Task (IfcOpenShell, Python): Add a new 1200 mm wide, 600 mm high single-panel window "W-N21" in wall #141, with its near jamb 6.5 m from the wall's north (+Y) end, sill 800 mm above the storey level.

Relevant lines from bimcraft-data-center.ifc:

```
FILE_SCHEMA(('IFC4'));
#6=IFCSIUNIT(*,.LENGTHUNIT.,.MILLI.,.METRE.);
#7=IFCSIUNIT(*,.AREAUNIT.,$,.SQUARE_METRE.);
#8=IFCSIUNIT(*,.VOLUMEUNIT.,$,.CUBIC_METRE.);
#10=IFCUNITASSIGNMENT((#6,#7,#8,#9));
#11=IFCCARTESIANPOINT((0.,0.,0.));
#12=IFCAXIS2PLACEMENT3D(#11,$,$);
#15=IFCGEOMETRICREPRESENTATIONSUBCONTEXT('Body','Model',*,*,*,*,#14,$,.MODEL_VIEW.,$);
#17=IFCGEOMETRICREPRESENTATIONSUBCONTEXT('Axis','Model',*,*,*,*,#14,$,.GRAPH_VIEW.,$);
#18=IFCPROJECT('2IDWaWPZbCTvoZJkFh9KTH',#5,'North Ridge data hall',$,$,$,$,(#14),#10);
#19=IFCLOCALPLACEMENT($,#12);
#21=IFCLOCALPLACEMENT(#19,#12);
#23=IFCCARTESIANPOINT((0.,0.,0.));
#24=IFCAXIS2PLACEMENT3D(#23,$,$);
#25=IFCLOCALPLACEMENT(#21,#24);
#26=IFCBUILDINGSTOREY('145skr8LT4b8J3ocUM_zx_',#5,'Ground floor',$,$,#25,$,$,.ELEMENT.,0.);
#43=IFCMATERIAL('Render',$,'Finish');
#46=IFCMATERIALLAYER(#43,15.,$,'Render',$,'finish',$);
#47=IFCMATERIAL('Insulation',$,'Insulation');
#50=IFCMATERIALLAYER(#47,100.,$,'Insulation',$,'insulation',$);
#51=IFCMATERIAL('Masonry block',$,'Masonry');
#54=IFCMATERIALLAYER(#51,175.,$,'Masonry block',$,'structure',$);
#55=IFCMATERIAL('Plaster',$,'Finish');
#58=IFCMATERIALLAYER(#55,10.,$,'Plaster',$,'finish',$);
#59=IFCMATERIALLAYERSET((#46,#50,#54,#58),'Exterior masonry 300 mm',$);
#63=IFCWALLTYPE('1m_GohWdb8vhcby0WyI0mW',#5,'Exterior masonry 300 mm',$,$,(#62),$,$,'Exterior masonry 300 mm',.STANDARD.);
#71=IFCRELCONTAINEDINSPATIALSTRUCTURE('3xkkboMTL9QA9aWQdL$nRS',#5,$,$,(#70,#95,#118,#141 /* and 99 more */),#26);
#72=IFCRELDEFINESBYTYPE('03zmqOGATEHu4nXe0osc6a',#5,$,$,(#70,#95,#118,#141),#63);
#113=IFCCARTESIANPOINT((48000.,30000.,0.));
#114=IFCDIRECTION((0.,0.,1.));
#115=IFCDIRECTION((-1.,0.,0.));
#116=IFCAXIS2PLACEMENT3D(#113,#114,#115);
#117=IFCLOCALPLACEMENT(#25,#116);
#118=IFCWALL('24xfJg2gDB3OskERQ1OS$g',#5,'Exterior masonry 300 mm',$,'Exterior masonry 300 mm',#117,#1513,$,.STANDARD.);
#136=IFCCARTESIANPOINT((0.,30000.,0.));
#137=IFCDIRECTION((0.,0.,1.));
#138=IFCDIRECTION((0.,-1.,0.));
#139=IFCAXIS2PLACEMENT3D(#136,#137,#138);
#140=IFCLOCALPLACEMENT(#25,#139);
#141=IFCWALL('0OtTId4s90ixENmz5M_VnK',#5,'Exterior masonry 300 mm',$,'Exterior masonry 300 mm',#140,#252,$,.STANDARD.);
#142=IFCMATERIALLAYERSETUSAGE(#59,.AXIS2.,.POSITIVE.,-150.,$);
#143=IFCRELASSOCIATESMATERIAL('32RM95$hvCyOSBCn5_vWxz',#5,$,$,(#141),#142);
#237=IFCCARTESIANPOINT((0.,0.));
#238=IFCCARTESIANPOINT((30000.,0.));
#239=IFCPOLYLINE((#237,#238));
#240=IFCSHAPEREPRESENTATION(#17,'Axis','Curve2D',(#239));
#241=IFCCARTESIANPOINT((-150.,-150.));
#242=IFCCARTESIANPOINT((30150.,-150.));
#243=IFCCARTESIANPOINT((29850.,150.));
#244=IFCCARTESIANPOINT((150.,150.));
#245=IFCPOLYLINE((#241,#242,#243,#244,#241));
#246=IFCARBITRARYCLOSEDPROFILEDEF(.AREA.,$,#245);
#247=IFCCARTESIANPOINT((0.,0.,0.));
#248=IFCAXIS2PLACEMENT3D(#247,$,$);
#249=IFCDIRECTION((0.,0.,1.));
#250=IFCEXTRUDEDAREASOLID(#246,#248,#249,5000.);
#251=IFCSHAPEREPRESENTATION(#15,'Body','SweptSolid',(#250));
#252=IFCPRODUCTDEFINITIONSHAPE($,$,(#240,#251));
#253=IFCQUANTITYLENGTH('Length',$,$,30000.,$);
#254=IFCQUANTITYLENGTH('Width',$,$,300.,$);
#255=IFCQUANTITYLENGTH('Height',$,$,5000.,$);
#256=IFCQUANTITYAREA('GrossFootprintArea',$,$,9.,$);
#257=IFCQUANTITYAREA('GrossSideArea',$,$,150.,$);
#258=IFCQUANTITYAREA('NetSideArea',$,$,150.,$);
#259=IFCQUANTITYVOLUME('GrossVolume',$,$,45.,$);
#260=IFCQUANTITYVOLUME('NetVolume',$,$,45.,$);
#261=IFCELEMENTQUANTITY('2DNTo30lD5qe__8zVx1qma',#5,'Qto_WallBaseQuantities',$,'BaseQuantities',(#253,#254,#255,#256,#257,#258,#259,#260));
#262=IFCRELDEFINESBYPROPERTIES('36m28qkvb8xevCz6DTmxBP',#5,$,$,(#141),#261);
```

```python
import numpy as np
import ifcopenshell
import ifcopenshell.api.feature
import ifcopenshell.api.geometry
import ifcopenshell.api.pset
import ifcopenshell.api.root
import ifcopenshell.api.spatial
import ifcopenshell.geom
import ifcopenshell.util.element
import ifcopenshell.util.placement
import ifcopenshell.util.representation
import ifcopenshell.util.shape
import ifcopenshell.util.unit

model = ifcopenshell.open("bimcraft-data-center.ifc")
unit_scale = ifcopenshell.util.unit.calculate_unit_scale(model)
area_scale = ifcopenshell.util.unit.calculate_unit_scale(model, "AREAUNIT")
volume_scale = ifcopenshell.util.unit.calculate_unit_scale(model, "VOLUMEUNIT")
settings = ifcopenshell.geom.settings()


def volume(element):
    """Net volume in cubic metres, openings subtracted."""
    shape = ifcopenshell.geom.create_shape(settings, element)
    return ifcopenshell.util.shape.get_volume(shape.geometry)


wall = model.by_id(141)
storey = ifcopenshell.util.element.get_container(wall, ifc_class="IfcBuildingStorey")
context = ifcopenshell.util.representation.get_context(model, "Model", "Body", "MODEL_VIEW")
before = volume(wall)

width, height, from_end, sill = 1.2, 0.6, 6.5, 0.8  # metres

# The wall runs along its own X axis, and the end named is its -X end.
wall_shape = ifcopenshell.geom.create_shape(settings, wall)
x, y, z = ifcopenshell.util.shape.get_vertices(wall_shape.geometry).T
start = x.min() + from_end
face, thickness = float(y.min()), float(y.max() - y.min())
wall_matrix = ifcopenshell.util.placement.get_local_placement(wall.ObjectPlacement)
level = ifcopenshell.util.placement.get_local_placement(storey.ObjectPlacement)[2, 3]


def in_wall(x, y):
    """Placement at x, y metres in the wall's axes, at sill height."""
    matrix = wall_matrix.copy()
    matrix[:, 3] = wall_matrix @ np.array([x / unit_scale, y / unit_scale, 0.0, 1.0])
    matrix[2, 3] = level + sill / unit_scale
    return matrix


# Opening: a box that overshoots both wall faces by 50 mm.
opening = ifcopenshell.api.root.create_entity(model, ifc_class="IfcOpeningElement", predefined_type="OPENING")
box = ifcopenshell.api.geometry.add_wall_representation(
    model, context=context, length=width, height=height, thickness=thickness + 0.1
)
ifcopenshell.api.geometry.assign_representation(model, product=opening, representation=box)
ifcopenshell.api.geometry.edit_object_placement(model, product=opening, matrix=in_wall(start, face - 0.05), is_si=False)
ifcopenshell.api.feature.add_feature(model, feature=opening, element=wall)

window = ifcopenshell.api.root.create_entity(model, ifc_class="IfcWindow", name="W-N21", predefined_type="WINDOW")
window.OverallWidth, window.OverallHeight = width / unit_scale, height / unit_scale
window.PartitioningType = "SINGLE_PANEL"
body = ifcopenshell.api.geometry.add_window_representation(
    model,
    context=context,
    overall_width=window.OverallWidth,
    overall_height=window.OverallHeight,
    partition_type="SINGLE_PANEL",
)
ifcopenshell.api.geometry.assign_representation(model, product=window, representation=body)
ifcopenshell.api.spatial.assign_container(model, products=[window], relating_structure=storey)
ifcopenshell.api.feature.add_filling(model, opening=opening, element=window)

# Centre the window in the wall's thickness.
ifcopenshell.api.geometry.edit_object_placement(model, product=window, matrix=in_wall(start, face), is_si=False)
window_shape = ifcopenshell.geom.create_shape(settings, window)
depth = ifcopenshell.util.shape.get_vertices(window_shape.geometry)[:, 1]
offset = face + thickness / 2 - (depth.min() + depth.max()) / 2
ifcopenshell.api.geometry.edit_object_placement(model, product=window, matrix=in_wall(start, offset), is_si=False)

after = volume(wall)

# Update the wall's stored quantities.
qto = model.by_id(ifcopenshell.util.element.get_pset(wall, "Qto_WallBaseQuantities", should_inherit=False)["id"])
ifcopenshell.api.pset.edit_qto(model, qto=qto, properties={
    "NetSideArea": after / thickness / area_scale,
    "NetVolume": after / volume_scale,
})

print(f"wall volume {before:.3f} -> {after:.3f} m3")

model.write("bimcraft-data-center-out.ifc")
```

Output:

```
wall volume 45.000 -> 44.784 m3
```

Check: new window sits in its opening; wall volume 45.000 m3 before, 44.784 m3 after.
